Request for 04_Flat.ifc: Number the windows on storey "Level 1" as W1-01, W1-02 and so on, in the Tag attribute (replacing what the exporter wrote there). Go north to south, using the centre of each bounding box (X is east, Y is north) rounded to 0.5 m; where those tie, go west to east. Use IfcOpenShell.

First a look at what the model holds.

```python
import ifcopenshell
import ifcopenshell.util.element
import ifcopenshell.util.placement

model = ifcopenshell.open("04_Flat.ifc")
print(model.schema)
storey = next(s for s in model.by_type("IfcBuildingStorey") if s.Name == "Level 1")
windows = [e for e in ifcopenshell.util.element.get_decomposition(storey) if e.is_a("IfcWindow")]
for e in sorted(windows, key=lambda e: e.id()):
    origin = ifcopenshell.util.placement.get_local_placement(e.ObjectPlacement)[:3, 3]
    print(e.id(), e.Tag, e.Name, origin.round(2) + 0.0, sep=" | ")
```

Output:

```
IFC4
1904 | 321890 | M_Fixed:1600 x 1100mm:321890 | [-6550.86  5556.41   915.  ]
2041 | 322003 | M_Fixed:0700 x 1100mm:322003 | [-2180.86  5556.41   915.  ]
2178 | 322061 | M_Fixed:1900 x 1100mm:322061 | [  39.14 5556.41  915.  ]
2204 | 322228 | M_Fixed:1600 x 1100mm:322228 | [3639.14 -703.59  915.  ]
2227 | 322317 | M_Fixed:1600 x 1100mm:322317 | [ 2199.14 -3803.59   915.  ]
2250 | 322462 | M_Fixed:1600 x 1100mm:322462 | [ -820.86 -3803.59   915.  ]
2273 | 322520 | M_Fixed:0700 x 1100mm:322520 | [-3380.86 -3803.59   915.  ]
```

```python
import ifcopenshell
import ifcopenshell.geom
import ifcopenshell.util.element
import ifcopenshell.util.shape

model = ifcopenshell.open("04_Flat.ifc")
settings = ifcopenshell.geom.settings()
settings.set("use-world-coords", True)


def centre(element):
    shape = ifcopenshell.geom.create_shape(settings, element)
    return ifcopenshell.util.shape.get_bbox_centroid(shape.geometry)


storey = next(s for s in model.by_type("IfcBuildingStorey") if s.Name == "Level 1")
windows = [e for e in ifcopenshell.util.element.get_decomposition(storey) if e.is_a("IfcWindow")]

# Insertion points can sit at a corner or the storey origin, so sort by the geometry (in metres).
centres = {e: centre(e) for e in windows}
windows.sort(key=lambda e: (-round(centres[e][1] / 0.5), centres[e][0]))

for i, e in enumerate(windows, start=1):
    number = f"W1-{i:02d}"
    e.Tag = number
    print(e.id(), number)

model.write("04_Flat_edited.ifc")
```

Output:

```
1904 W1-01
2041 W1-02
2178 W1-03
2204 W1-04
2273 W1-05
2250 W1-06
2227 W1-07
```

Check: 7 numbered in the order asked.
